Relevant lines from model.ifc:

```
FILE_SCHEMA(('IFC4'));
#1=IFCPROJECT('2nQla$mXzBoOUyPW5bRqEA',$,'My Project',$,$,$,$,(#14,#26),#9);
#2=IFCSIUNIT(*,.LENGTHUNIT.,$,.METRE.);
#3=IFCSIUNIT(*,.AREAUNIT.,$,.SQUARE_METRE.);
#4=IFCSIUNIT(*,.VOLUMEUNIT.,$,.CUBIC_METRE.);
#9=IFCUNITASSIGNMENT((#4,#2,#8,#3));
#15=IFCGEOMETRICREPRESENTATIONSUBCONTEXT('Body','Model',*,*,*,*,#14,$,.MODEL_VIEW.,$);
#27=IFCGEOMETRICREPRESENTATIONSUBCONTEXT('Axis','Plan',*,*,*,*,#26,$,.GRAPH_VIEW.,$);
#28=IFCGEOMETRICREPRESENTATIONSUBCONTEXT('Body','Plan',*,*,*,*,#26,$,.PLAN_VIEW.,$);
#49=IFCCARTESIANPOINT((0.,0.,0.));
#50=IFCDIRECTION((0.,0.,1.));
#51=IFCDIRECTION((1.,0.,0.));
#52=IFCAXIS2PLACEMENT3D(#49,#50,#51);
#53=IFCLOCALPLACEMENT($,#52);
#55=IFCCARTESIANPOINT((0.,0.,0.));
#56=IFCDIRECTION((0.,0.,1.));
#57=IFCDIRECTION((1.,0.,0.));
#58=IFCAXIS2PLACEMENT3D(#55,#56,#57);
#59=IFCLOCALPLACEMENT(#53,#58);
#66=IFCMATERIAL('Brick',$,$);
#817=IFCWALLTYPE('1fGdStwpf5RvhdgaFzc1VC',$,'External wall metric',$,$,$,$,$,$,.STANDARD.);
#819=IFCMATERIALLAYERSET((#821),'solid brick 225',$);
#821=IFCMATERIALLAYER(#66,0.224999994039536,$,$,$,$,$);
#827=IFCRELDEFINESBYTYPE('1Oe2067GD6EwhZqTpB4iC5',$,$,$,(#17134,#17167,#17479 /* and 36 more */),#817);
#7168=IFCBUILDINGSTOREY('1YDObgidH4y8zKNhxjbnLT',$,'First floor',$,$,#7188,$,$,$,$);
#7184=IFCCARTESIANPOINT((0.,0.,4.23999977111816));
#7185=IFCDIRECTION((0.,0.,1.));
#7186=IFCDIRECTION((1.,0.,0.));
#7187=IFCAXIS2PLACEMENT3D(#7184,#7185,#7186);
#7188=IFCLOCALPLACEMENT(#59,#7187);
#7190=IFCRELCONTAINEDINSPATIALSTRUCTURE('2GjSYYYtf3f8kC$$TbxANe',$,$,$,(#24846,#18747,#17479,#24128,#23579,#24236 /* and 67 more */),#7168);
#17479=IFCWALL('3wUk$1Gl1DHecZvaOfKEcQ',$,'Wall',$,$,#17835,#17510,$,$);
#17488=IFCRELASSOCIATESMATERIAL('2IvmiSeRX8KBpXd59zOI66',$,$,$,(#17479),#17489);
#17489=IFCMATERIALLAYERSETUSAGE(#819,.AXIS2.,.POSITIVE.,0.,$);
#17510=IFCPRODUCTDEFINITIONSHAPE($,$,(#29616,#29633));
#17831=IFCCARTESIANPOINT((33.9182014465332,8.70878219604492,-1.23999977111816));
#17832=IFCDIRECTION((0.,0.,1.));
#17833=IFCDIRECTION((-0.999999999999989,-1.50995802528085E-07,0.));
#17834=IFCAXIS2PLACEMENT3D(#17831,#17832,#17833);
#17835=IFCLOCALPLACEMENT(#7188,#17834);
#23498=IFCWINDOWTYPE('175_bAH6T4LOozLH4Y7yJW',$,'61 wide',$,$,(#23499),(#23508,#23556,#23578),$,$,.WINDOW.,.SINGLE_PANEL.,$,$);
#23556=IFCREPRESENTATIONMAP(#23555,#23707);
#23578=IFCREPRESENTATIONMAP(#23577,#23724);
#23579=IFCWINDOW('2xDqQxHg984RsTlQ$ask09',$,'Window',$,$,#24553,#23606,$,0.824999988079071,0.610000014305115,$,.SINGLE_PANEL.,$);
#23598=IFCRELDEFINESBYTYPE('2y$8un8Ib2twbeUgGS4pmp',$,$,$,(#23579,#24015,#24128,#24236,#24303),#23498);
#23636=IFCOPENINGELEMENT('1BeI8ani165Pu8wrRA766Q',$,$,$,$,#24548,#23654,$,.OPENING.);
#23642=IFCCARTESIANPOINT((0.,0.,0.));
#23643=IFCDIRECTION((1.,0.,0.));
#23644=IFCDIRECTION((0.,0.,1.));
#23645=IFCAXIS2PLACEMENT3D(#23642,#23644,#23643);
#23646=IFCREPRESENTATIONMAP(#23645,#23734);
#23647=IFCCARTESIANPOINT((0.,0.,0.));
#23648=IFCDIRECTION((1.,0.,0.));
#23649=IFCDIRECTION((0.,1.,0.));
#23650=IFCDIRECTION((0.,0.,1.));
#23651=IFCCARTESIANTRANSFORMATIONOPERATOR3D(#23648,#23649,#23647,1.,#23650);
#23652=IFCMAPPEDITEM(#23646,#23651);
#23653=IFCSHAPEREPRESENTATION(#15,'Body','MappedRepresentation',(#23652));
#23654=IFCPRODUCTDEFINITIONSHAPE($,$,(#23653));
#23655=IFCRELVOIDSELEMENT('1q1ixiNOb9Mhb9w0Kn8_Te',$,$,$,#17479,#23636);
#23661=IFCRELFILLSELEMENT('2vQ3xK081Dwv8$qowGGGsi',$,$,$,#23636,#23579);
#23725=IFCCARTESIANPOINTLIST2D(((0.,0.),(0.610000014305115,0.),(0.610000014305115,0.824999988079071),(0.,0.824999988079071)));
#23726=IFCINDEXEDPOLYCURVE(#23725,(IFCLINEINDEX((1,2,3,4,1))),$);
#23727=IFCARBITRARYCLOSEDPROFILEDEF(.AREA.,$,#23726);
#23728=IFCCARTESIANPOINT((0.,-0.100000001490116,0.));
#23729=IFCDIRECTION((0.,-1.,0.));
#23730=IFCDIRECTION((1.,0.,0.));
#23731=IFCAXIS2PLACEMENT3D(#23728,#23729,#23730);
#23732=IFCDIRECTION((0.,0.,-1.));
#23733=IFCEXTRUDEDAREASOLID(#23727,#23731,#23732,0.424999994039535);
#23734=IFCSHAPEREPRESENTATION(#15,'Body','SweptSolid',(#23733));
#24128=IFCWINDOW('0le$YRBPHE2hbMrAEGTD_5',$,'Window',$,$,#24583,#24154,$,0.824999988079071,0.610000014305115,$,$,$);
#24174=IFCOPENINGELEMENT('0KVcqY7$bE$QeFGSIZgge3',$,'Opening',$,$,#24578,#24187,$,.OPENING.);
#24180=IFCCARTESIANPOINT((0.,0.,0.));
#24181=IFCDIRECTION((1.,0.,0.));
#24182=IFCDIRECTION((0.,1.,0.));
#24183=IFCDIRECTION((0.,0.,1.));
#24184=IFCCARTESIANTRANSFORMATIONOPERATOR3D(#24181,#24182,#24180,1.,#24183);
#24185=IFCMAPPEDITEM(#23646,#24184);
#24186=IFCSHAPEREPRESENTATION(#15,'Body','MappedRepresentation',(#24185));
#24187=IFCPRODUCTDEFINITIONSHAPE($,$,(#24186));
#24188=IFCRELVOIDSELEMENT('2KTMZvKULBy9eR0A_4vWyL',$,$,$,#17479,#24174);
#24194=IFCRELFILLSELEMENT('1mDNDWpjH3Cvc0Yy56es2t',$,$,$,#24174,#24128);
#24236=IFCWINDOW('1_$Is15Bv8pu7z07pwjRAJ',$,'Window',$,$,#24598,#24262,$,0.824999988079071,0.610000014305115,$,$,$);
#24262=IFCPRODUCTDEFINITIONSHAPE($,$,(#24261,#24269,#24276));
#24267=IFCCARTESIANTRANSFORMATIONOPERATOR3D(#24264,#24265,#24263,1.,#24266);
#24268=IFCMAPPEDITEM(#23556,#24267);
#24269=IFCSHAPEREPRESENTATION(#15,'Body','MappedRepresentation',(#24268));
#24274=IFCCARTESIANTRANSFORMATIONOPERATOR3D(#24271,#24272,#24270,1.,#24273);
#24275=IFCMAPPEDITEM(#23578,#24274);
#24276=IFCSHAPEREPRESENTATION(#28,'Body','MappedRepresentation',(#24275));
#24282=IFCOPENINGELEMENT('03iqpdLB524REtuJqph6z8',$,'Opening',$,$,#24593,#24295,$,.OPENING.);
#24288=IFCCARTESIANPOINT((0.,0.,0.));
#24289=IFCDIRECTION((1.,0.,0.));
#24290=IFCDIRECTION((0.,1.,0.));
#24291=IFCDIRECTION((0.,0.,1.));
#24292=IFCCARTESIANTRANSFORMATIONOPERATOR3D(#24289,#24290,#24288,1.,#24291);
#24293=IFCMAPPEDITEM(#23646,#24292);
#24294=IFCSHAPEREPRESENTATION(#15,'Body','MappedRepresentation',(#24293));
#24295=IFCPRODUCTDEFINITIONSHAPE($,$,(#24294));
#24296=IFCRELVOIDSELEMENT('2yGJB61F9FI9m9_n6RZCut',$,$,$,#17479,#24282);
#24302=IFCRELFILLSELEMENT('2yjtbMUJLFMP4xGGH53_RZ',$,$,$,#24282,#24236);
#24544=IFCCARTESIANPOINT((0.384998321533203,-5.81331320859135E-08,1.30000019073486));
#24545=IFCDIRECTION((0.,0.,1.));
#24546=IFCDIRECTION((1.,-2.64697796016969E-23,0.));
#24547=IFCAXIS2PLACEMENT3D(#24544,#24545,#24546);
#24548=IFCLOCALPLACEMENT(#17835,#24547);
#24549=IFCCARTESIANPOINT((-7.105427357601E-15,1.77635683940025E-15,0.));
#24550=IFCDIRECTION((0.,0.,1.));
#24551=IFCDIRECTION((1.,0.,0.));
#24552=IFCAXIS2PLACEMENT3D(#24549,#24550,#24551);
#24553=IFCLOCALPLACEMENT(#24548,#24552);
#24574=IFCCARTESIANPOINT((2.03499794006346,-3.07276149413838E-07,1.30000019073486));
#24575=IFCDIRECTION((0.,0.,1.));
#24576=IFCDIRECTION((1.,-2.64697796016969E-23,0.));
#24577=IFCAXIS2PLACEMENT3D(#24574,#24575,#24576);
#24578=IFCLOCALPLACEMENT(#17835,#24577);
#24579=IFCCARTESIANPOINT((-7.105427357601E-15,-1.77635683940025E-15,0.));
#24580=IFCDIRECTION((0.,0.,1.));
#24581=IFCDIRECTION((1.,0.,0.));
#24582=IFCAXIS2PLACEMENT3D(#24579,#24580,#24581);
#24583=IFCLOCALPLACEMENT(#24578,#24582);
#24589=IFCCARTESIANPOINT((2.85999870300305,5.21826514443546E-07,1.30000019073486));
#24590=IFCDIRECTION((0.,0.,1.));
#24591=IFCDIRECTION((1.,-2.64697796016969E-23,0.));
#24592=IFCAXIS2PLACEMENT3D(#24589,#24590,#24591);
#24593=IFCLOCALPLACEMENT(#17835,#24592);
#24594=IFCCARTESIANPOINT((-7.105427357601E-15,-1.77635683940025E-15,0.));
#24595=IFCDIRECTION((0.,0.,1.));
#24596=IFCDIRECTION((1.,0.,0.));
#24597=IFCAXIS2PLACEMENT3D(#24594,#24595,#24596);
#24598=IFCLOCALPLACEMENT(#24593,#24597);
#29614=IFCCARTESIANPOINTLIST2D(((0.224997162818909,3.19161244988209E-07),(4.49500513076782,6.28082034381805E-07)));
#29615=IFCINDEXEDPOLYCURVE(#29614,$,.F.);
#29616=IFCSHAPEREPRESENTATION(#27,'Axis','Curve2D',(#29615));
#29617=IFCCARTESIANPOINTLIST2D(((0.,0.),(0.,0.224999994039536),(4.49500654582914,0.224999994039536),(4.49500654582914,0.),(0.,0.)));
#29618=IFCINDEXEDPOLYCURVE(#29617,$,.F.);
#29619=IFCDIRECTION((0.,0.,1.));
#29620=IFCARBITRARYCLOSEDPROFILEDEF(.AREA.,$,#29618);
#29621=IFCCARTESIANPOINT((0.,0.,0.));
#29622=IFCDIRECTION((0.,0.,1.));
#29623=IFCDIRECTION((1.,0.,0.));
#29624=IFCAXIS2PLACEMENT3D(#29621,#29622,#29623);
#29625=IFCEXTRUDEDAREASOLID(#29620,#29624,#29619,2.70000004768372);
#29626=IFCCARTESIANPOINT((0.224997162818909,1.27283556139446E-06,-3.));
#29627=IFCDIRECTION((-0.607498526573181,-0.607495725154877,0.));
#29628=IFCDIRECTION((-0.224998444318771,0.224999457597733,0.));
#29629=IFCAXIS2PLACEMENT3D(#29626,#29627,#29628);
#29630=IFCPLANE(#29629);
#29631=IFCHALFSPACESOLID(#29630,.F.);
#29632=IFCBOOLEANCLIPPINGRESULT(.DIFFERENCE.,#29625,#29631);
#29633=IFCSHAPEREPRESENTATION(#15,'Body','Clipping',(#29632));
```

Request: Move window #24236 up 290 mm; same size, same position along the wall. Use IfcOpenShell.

```python
import numpy as np
import ifcopenshell
import ifcopenshell.api.geometry
import ifcopenshell.util.placement
import ifcopenshell.util.unit

model = ifcopenshell.open("model.ifc")
unit_scale = ifcopenshell.util.unit.calculate_unit_scale(model)

window = model.by_guid("1_$Is15Bv8pu7z07pwjRAJ")
opening = window.FillsVoids[0].RelatingOpeningElement
dz = 0.29

shift = np.array([0.0, 0.0, dz])
# The window is placed relative to its opening, so it follows when the opening moves.
matrix = ifcopenshell.util.placement.get_local_placement(opening.ObjectPlacement)
matrix[:3, 3] += shift
ifcopenshell.api.geometry.edit_object_placement(
    model, product=opening, matrix=matrix, is_si=False, should_transform_children=True
)

print(f"moved by {dz * unit_scale:+.3f} m")

model.write("model_updated.ifc")
```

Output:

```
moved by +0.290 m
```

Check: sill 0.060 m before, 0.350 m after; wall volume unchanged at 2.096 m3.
